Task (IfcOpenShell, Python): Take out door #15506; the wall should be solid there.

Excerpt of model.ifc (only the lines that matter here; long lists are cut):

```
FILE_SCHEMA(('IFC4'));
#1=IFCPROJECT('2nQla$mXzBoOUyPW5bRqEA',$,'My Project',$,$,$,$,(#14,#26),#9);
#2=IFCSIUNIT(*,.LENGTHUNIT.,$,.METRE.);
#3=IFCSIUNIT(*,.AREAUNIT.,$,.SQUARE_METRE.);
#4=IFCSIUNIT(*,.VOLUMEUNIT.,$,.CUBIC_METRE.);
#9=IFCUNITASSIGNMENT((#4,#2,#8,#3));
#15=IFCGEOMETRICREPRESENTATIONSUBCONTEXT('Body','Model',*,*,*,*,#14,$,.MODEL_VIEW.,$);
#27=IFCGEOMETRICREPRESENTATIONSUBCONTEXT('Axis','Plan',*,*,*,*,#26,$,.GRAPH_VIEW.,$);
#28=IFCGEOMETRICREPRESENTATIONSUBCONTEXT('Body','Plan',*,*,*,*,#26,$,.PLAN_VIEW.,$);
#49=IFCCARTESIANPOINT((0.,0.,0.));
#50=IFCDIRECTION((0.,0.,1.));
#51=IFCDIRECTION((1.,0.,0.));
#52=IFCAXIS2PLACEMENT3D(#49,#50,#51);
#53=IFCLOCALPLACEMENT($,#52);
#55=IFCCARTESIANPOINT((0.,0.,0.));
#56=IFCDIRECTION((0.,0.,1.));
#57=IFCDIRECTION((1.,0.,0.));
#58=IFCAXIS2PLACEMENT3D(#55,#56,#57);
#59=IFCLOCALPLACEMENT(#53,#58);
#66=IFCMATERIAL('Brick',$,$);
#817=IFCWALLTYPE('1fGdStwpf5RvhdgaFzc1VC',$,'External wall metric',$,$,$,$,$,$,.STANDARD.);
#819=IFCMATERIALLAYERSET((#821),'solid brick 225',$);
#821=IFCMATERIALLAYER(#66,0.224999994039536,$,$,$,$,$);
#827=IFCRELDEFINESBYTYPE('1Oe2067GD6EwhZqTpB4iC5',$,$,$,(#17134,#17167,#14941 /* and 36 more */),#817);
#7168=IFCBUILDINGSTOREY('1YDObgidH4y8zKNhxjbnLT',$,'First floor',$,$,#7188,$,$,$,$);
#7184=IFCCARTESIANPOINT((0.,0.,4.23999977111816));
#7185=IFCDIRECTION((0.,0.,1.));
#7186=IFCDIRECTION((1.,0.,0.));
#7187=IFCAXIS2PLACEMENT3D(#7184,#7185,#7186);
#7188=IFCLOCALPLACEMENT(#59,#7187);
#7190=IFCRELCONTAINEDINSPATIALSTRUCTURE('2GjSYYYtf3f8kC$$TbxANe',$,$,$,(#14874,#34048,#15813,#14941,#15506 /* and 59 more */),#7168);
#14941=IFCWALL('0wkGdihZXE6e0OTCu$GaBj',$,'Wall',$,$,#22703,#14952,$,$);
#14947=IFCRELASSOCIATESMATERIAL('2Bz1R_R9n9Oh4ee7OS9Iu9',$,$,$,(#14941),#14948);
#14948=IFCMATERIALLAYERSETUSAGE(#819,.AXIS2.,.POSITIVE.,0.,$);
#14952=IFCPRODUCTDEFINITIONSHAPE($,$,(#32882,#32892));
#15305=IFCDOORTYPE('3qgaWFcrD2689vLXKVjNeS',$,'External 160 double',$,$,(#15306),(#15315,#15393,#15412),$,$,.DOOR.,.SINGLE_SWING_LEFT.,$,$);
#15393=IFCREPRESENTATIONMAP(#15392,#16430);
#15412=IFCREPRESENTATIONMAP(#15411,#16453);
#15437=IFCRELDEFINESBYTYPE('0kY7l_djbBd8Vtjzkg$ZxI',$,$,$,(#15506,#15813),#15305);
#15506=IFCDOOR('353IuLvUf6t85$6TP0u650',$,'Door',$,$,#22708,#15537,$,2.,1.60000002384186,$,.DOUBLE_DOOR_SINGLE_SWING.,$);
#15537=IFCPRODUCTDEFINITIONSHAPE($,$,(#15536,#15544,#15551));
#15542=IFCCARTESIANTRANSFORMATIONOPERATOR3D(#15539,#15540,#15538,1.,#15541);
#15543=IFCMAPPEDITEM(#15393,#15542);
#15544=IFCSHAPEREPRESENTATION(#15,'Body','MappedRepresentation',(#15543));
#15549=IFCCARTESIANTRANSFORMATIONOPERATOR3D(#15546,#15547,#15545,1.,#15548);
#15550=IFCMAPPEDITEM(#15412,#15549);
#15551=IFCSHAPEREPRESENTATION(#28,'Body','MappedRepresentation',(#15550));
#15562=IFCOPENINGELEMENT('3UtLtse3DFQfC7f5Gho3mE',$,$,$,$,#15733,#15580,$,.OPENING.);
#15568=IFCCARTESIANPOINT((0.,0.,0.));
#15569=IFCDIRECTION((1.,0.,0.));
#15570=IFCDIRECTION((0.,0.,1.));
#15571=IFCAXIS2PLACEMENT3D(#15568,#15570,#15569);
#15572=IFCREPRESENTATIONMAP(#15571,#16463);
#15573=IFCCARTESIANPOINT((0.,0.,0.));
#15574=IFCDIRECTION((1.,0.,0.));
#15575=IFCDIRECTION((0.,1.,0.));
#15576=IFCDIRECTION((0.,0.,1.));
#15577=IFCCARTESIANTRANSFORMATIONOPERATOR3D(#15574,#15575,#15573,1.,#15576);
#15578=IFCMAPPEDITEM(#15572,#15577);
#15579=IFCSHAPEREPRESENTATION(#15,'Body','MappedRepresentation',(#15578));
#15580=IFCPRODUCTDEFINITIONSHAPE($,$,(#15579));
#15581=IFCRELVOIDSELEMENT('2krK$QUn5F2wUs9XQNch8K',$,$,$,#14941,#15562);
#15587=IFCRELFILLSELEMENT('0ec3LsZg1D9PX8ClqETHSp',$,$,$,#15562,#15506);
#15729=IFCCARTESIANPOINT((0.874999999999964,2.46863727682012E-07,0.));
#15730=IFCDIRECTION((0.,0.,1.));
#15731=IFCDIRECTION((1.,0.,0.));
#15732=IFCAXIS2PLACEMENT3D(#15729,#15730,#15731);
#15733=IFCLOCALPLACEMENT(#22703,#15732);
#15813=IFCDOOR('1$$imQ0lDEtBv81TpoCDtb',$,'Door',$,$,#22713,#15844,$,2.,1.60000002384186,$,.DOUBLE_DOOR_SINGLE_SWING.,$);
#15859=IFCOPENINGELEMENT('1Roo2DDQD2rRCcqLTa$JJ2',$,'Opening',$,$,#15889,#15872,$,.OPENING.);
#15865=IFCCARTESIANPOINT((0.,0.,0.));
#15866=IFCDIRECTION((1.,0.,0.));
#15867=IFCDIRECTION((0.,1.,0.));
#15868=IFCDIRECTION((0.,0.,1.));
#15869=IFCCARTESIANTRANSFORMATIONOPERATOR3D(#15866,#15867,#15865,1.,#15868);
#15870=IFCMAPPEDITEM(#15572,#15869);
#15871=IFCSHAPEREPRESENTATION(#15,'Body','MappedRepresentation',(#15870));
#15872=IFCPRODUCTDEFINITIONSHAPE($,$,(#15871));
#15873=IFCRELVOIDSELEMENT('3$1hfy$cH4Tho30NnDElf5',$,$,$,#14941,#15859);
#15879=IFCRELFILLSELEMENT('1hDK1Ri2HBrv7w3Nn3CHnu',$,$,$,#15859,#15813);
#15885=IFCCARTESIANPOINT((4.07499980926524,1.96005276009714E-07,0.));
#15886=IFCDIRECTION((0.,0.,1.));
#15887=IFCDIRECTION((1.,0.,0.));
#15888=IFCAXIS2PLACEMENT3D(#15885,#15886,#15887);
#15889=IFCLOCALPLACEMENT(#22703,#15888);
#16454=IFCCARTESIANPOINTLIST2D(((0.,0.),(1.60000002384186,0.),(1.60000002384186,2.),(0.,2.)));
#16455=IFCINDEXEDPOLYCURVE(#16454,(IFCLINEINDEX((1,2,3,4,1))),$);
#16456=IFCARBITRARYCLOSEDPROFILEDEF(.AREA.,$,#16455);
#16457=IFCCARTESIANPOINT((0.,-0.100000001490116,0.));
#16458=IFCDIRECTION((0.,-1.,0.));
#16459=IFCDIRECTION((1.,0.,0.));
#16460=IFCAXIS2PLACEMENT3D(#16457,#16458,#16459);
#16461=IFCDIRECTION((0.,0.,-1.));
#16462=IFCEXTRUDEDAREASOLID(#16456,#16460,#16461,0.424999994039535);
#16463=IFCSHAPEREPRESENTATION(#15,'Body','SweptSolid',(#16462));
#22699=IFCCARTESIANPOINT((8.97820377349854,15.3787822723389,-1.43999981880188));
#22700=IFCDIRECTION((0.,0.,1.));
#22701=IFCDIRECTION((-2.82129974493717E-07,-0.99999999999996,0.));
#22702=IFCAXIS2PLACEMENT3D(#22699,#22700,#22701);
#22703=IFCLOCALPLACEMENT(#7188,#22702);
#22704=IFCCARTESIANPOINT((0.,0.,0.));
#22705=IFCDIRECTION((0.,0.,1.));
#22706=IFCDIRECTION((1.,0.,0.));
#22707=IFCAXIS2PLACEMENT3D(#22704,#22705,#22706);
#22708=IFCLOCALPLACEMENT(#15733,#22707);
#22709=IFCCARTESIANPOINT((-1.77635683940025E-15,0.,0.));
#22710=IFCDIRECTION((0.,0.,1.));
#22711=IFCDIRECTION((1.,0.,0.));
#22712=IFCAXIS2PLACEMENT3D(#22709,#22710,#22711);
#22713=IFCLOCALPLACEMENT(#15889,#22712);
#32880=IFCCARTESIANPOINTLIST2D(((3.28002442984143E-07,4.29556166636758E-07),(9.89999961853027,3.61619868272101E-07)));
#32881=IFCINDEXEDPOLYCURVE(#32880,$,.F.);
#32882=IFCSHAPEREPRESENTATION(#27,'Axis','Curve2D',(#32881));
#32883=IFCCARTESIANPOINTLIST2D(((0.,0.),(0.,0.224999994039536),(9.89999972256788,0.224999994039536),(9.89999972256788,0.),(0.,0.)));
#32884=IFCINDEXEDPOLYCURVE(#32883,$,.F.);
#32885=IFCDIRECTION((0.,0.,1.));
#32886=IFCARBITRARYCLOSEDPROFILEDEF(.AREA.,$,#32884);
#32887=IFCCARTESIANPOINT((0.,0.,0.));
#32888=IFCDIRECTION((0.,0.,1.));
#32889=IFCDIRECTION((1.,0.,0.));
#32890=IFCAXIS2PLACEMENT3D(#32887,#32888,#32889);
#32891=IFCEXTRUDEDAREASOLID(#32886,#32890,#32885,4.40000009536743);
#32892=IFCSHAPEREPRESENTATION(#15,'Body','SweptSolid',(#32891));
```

```python
import ifcopenshell
import ifcopenshell.api.feature
import ifcopenshell.api.root
import ifcopenshell.geom
import ifcopenshell.util.shape

model = ifcopenshell.open("model.ifc")
settings = ifcopenshell.geom.settings()


def volume(element):
    """Net volume in cubic metres, openings subtracted."""
    shape = ifcopenshell.geom.create_shape(settings, element)
    return ifcopenshell.util.shape.get_volume(shape.geometry)


door = model.by_id(15506)
opening = door.FillsVoids[0].RelatingOpeningElement
wall = opening.VoidsElements[0].RelatingBuildingElement
before = volume(wall)

ifcopenshell.api.root.remove_product(model, product=door)
ifcopenshell.api.feature.remove_feature(model, feature=opening)

after = volume(wall)

print(f"wall volume {before:.3f} -> {after:.3f} m3")

model.write("model_edited.ifc")
```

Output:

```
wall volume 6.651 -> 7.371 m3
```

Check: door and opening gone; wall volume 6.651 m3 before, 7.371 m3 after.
